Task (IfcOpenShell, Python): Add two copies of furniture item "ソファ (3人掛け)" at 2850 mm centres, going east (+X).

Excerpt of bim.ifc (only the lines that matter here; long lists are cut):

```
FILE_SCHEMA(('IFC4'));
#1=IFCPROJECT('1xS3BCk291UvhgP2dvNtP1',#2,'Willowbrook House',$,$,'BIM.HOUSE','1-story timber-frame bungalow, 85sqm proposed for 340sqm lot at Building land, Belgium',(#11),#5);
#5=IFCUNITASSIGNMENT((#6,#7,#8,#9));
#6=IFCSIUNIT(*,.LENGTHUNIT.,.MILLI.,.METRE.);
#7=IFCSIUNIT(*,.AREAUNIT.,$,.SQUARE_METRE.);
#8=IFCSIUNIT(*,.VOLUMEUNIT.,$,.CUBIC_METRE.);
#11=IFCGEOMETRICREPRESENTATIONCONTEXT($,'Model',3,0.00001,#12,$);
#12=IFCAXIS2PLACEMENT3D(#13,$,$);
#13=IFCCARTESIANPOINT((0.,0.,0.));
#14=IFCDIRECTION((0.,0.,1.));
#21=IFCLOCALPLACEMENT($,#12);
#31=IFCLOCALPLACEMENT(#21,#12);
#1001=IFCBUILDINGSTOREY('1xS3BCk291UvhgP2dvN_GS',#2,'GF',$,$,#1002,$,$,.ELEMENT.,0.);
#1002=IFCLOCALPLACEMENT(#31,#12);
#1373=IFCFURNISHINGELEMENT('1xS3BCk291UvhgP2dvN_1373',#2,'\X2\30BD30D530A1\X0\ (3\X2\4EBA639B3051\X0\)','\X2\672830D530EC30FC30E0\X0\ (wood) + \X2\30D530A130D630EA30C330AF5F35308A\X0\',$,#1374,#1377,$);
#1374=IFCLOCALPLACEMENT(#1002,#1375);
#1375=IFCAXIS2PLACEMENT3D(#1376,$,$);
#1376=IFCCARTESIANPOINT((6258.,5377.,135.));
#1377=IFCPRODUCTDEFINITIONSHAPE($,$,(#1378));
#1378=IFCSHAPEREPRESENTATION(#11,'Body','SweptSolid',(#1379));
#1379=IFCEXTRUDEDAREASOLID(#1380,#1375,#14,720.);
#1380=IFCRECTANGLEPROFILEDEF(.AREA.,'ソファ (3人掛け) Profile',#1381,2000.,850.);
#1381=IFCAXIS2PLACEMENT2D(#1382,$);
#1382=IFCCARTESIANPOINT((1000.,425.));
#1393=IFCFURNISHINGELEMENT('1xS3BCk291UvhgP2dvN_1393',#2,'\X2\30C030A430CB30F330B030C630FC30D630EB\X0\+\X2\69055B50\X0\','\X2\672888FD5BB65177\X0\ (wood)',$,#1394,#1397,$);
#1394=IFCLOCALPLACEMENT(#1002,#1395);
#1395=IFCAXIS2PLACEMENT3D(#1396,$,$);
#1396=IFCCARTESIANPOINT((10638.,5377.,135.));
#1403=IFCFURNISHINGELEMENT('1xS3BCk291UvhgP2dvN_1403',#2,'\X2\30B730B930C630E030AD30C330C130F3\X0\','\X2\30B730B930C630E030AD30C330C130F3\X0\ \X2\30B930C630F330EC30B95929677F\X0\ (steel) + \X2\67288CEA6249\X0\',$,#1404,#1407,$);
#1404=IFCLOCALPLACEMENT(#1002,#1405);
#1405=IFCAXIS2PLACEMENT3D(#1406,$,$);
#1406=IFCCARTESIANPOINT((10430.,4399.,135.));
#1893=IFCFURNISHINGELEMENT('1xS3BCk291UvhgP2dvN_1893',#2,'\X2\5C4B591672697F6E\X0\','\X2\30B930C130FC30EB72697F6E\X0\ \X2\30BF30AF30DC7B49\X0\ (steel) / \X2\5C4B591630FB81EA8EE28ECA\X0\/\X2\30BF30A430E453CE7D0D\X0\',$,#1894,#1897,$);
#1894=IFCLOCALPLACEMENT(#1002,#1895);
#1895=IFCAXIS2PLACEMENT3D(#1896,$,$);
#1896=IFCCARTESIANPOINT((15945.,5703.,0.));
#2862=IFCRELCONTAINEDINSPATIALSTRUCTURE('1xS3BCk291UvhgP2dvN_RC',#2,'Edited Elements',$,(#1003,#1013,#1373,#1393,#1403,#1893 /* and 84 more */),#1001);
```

```python
import numpy as np
import ifcopenshell
import ifcopenshell.api.geometry
import ifcopenshell.api.root
import ifcopenshell.util.element
import ifcopenshell.util.placement
import ifcopenshell.util.unit

model = ifcopenshell.open("bim.ifc")
unit_scale = ifcopenshell.util.unit.calculate_unit_scale(model)


def reuse_history(source, copy):
    """copy_class also copies each property set's owner history, people and application; keep the originals."""
    for rel in copy.IsDefinedBy:
        if rel.is_a("IfcRelDefinesByProperties") and (history := rel.RelatingPropertyDefinition.OwnerHistory):
            rel.RelatingPropertyDefinition.OwnerHistory = source.OwnerHistory
            ifcopenshell.util.element.remove_deep2(model, history)


source = model.by_id(1373)
base = ifcopenshell.util.placement.get_local_placement(source.ObjectPlacement)
step = np.array([1.0, 0.0, 0.0]) * 2.85 / unit_scale

for i in range(1, 3):
    copy = ifcopenshell.api.root.copy_class(model, product=source)
    copy.Representation = ifcopenshell.util.element.copy_deep(
        model, source.Representation, exclude=["IfcGeometricRepresentationContext", "IfcRepresentationMap"]
    )
    reuse_history(source, copy)
    matrix = base.copy()
    matrix[:3, 3] += i * step
    print("added at", matrix[:3, 3].round(3) + 0.0)
    ifcopenshell.api.geometry.edit_object_placement(model, product=copy, matrix=matrix, is_si=False)

model.write("bim_rev.ifc")
```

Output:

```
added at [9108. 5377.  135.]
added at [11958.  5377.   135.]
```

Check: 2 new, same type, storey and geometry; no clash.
